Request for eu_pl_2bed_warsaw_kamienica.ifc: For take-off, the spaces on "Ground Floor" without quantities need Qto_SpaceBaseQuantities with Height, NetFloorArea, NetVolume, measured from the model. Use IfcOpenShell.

First a look at what the model holds.

```python
import ifcopenshell
import ifcopenshell.util.element
import ifcopenshell.util.unit

model = ifcopenshell.open("eu_pl_2bed_warsaw_kamienica.ifc")
print(model.schema)
for unit_type in ("LENGTHUNIT", "AREAUNIT", "VOLUMEUNIT"):
    print(unit_type, ifcopenshell.util.unit.calculate_unit_scale(model, unit_type))
storey = next(s for s in model.by_type("IfcBuildingStorey") if s.Name == "Ground Floor")
spaces = [e for e in ifcopenshell.util.element.get_decomposition(storey) if e.is_a("IfcSpace")]
for e in sorted(spaces, key=lambda e: e.id()):
    print(e.id(), e.is_a(), e.Name, list(ifcopenshell.util.element.get_psets(e, qtos_only=True)), sep=" | ")
```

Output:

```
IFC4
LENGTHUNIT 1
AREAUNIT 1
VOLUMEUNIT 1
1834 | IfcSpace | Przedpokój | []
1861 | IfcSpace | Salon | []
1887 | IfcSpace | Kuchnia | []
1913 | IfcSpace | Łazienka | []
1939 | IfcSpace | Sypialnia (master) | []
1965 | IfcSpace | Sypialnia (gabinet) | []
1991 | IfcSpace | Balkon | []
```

```python
import ifcopenshell
import ifcopenshell.api.pset
import ifcopenshell.geom
import ifcopenshell.util.element
import ifcopenshell.util.shape
import ifcopenshell.util.unit

model = ifcopenshell.open("eu_pl_2bed_warsaw_kamienica.ifc")
unit_scale = ifcopenshell.util.unit.calculate_unit_scale(model)
area_scale = ifcopenshell.util.unit.calculate_unit_scale(model, "AREAUNIT")
volume_scale = ifcopenshell.util.unit.calculate_unit_scale(model, "VOLUMEUNIT")
settings = ifcopenshell.geom.settings()

storey = next(s for s in model.by_type("IfcBuildingStorey") if s.Name == "Ground Floor")
spaces = [e for e in ifcopenshell.util.element.get_decomposition(storey) if e.is_a("IfcSpace")]

for e in sorted(spaces, key=lambda e: e.id()):
    if ifcopenshell.util.element.get_psets(e, qtos_only=True, should_inherit=False):
        continue
    # Geometry comes back in metres, in the element's own axes.
    shape = ifcopenshell.geom.create_shape(settings, e)
    values = {
        "Height": ifcopenshell.util.shape.get_z(shape.geometry) / unit_scale,
        "NetFloorArea": ifcopenshell.util.shape.get_footprint_area(shape.geometry) / area_scale,
        "NetVolume": ifcopenshell.util.shape.get_volume(shape.geometry) / volume_scale,
    }
    qto = ifcopenshell.api.pset.add_qto(model, product=e, name="Qto_SpaceBaseQuantities")
    ifcopenshell.api.pset.edit_qto(model, qto=qto, properties=values)
    print(e.id(), {k: round(v, 3) for k, v in values.items()})

model.write("eu_pl_2bed_warsaw_kamienica_edited.ifc")
```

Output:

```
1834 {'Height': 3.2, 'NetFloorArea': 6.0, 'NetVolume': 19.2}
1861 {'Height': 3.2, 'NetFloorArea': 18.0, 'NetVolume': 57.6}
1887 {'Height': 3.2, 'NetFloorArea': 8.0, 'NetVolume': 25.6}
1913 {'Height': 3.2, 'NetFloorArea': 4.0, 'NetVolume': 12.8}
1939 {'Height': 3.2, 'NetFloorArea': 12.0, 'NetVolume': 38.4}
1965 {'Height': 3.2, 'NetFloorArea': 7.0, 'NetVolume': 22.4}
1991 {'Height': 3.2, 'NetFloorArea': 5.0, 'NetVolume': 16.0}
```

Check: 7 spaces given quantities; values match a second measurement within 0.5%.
